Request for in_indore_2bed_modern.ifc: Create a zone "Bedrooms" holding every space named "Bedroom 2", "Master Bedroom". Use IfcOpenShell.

First a look at what the model holds.

```python
import ifcopenshell

model = ifcopenshell.open("in_indore_2bed_modern.ifc")
print(model.schema)
seen = {}
for space in model.by_type("IfcSpace"):
    seen[space.LongName] = seen.get(space.LongName, 0) + 1
for name, count in sorted(seen.items(), key=str):
    print(count, "x", name)
print("zones:", [z.Name for z in model.by_type("IfcZone")][:20])
```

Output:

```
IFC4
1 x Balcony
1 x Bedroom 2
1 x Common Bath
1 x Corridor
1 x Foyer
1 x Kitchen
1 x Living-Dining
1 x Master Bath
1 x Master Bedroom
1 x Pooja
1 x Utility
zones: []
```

```python
import ifcopenshell
import ifcopenshell.api.group
import ifcopenshell.api.root

model = ifcopenshell.open("in_indore_2bed_modern.ifc")

names = {"Bedroom 2", "Master Bedroom"}
spaces = [s for s in model.by_type("IfcSpace") if s.LongName in names]

zone = ifcopenshell.api.root.create_entity(model, ifc_class="IfcZone", name="Bedrooms")
ifcopenshell.api.group.assign_group(model, products=spaces, group=zone)
print(len(spaces), "spaces in", zone.Name)

model.write("in_indore_2bed_modern_edited.ifc")
```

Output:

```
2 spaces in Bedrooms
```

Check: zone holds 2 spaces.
